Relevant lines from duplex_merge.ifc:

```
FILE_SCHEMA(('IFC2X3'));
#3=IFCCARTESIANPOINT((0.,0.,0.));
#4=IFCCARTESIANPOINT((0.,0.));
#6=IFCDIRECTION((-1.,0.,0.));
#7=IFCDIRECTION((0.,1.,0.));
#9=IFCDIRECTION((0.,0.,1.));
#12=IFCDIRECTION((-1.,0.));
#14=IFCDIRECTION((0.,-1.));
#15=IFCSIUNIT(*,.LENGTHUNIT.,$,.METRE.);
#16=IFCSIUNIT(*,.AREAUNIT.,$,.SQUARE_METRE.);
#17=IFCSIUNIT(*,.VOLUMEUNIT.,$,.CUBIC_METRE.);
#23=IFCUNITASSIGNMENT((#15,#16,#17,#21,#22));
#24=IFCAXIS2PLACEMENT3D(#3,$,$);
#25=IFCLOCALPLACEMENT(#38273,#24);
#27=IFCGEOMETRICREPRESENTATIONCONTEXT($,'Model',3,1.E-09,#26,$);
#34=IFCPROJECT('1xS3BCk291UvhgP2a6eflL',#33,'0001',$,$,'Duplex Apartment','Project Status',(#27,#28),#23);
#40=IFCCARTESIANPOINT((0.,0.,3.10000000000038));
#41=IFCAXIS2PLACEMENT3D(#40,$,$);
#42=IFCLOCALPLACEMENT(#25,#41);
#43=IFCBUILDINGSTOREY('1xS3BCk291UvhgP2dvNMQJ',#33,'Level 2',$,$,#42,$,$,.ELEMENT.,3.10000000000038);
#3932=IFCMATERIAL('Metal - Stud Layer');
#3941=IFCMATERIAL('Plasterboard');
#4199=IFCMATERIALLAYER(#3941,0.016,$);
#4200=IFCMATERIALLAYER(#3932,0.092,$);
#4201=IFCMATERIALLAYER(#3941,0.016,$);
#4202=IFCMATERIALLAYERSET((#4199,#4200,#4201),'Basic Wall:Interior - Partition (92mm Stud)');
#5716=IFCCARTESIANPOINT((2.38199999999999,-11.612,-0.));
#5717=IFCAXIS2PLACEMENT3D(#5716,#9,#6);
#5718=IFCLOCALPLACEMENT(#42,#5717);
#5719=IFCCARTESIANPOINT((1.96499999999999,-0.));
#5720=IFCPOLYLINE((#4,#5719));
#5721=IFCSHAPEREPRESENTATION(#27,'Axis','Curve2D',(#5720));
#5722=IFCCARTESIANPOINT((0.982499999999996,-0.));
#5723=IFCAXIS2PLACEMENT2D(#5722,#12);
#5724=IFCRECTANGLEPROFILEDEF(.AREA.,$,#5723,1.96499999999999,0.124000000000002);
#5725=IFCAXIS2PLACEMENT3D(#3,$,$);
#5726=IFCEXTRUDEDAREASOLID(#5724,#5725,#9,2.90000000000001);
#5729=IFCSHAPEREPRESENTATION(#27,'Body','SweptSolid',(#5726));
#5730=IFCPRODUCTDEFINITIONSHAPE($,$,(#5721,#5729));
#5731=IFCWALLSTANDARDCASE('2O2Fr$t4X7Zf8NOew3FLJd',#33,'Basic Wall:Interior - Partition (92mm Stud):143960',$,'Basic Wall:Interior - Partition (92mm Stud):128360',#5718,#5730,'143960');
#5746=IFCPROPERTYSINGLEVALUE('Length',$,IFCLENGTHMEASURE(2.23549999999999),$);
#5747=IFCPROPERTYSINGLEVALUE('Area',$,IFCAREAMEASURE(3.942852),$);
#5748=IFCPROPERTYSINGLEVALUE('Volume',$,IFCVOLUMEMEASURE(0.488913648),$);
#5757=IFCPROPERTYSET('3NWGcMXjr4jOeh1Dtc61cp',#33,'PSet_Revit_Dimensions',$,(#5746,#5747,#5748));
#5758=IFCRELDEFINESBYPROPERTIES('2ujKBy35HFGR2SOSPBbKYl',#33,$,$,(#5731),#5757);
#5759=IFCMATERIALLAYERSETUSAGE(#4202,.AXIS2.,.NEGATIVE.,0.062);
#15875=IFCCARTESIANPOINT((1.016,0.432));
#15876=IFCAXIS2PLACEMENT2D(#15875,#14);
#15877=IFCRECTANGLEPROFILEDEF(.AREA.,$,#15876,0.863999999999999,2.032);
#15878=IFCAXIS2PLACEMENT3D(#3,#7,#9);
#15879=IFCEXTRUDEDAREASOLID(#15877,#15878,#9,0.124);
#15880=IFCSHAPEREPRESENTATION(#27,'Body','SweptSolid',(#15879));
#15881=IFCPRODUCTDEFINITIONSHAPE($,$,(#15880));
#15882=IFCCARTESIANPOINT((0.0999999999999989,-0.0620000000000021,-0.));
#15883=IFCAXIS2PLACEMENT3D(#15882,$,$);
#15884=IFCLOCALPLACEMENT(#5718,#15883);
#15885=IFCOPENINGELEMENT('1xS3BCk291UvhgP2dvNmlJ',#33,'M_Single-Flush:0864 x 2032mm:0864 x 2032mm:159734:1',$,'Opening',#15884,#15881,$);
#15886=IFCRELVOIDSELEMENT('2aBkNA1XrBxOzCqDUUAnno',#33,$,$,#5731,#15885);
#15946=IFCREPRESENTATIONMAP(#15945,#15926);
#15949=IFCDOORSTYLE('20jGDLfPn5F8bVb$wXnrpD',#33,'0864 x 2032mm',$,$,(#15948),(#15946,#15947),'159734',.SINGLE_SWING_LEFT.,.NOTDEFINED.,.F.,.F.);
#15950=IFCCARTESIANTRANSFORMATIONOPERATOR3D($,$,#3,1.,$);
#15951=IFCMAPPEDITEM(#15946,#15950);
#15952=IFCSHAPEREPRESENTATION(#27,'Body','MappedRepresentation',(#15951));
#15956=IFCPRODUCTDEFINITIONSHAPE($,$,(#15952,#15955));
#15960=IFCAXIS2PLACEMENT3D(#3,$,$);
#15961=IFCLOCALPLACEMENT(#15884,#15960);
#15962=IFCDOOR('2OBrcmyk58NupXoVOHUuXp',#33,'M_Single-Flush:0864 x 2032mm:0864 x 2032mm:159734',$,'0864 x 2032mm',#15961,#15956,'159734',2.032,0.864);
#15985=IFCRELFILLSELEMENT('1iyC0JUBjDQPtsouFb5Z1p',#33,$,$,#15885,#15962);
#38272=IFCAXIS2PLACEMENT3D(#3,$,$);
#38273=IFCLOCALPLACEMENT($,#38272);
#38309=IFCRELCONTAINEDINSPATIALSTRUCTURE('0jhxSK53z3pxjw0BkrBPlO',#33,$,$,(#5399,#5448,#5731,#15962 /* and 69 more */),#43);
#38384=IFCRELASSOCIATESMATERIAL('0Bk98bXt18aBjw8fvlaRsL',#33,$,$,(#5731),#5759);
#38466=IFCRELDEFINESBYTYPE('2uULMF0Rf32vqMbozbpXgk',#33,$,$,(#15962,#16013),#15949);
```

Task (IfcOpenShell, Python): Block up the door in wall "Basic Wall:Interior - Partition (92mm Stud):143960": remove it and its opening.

```python
import ifcopenshell
import ifcopenshell.api.feature
import ifcopenshell.api.pset
import ifcopenshell.api.root
import ifcopenshell.geom
import ifcopenshell.util.element
import ifcopenshell.util.shape
import ifcopenshell.util.unit

model = ifcopenshell.open("duplex_merge.ifc")
area_scale = ifcopenshell.util.unit.calculate_unit_scale(model, "AREAUNIT")
volume_scale = ifcopenshell.util.unit.calculate_unit_scale(model, "VOLUMEUNIT")
settings = ifcopenshell.geom.settings()


def volume(element):
    """Net volume in cubic metres, openings subtracted."""
    shape = ifcopenshell.geom.create_shape(settings, element)
    return ifcopenshell.util.shape.get_volume(shape.geometry)


door = model.by_guid("2OBrcmyk58NupXoVOHUuXp")
opening = door.FillsVoids[0].RelatingOpeningElement
wall = opening.VoidsElements[0].RelatingBuildingElement
before = volume(wall)

ifcopenshell.api.root.remove_product(model, product=door)
ifcopenshell.api.feature.remove_feature(model, feature=opening)

after = volume(wall)
thickness = 0.124  # wall thickness in metres

# Update the wall's stored quantities.
pset = model.by_id(ifcopenshell.util.element.get_pset(wall, "PSet_Revit_Dimensions", should_inherit=False)["id"])
ifcopenshell.api.pset.edit_pset(model, pset=pset, properties={
    "Area": model.create_entity("IfcAreaMeasure", after / thickness / area_scale),
    "Volume": model.create_entity("IfcVolumeMeasure", after / volume_scale),
})

print(f"wall volume {before:.3f} -> {after:.3f} m3")

model.write("duplex_merge_updated.ifc")
```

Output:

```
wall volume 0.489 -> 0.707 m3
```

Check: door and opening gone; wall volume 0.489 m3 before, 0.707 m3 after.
